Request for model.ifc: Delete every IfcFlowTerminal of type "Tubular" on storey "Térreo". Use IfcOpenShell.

First a look at what the model holds.

```python
import ifcopenshell
import ifcopenshell.util.element

model = ifcopenshell.open("model.ifc")
print(model.schema)
storey = next(s for s in model.by_type("IfcBuildingStorey") if s.Name == "Térreo")
terminals = [e for e in ifcopenshell.util.element.get_decomposition(storey) if e.is_a("IfcFlowTerminal")]
seen = {}
for e in terminals:
    element_type = ifcopenshell.util.element.get_type(e)
    name = element_type.Name if element_type not in (None, e) else None
    seen[name] = seen.get(name, 0) + 1
for name, count in sorted(seen.items(), key=str):
    print(count, "x", name)
```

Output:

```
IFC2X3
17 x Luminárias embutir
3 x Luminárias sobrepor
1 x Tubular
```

```python
import ifcopenshell
import ifcopenshell.api.root
import ifcopenshell.util.element

model = ifcopenshell.open("model.ifc")

storey = next(s for s in model.by_type("IfcBuildingStorey") if s.Name == "Térreo")
terminals = [e for e in ifcopenshell.util.element.get_decomposition(storey) if e.is_a("IfcFlowTerminal")]
targets = [e for e in terminals if (t := ifcopenshell.util.element.get_type(e)) not in (None, e) and t.Name == "Tubular"]

for e in targets:
    ifcopenshell.api.root.remove_product(model, product=e)
print(len(targets), "removed")

model.write("model_v2.ifc")
```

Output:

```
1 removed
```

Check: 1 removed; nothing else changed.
